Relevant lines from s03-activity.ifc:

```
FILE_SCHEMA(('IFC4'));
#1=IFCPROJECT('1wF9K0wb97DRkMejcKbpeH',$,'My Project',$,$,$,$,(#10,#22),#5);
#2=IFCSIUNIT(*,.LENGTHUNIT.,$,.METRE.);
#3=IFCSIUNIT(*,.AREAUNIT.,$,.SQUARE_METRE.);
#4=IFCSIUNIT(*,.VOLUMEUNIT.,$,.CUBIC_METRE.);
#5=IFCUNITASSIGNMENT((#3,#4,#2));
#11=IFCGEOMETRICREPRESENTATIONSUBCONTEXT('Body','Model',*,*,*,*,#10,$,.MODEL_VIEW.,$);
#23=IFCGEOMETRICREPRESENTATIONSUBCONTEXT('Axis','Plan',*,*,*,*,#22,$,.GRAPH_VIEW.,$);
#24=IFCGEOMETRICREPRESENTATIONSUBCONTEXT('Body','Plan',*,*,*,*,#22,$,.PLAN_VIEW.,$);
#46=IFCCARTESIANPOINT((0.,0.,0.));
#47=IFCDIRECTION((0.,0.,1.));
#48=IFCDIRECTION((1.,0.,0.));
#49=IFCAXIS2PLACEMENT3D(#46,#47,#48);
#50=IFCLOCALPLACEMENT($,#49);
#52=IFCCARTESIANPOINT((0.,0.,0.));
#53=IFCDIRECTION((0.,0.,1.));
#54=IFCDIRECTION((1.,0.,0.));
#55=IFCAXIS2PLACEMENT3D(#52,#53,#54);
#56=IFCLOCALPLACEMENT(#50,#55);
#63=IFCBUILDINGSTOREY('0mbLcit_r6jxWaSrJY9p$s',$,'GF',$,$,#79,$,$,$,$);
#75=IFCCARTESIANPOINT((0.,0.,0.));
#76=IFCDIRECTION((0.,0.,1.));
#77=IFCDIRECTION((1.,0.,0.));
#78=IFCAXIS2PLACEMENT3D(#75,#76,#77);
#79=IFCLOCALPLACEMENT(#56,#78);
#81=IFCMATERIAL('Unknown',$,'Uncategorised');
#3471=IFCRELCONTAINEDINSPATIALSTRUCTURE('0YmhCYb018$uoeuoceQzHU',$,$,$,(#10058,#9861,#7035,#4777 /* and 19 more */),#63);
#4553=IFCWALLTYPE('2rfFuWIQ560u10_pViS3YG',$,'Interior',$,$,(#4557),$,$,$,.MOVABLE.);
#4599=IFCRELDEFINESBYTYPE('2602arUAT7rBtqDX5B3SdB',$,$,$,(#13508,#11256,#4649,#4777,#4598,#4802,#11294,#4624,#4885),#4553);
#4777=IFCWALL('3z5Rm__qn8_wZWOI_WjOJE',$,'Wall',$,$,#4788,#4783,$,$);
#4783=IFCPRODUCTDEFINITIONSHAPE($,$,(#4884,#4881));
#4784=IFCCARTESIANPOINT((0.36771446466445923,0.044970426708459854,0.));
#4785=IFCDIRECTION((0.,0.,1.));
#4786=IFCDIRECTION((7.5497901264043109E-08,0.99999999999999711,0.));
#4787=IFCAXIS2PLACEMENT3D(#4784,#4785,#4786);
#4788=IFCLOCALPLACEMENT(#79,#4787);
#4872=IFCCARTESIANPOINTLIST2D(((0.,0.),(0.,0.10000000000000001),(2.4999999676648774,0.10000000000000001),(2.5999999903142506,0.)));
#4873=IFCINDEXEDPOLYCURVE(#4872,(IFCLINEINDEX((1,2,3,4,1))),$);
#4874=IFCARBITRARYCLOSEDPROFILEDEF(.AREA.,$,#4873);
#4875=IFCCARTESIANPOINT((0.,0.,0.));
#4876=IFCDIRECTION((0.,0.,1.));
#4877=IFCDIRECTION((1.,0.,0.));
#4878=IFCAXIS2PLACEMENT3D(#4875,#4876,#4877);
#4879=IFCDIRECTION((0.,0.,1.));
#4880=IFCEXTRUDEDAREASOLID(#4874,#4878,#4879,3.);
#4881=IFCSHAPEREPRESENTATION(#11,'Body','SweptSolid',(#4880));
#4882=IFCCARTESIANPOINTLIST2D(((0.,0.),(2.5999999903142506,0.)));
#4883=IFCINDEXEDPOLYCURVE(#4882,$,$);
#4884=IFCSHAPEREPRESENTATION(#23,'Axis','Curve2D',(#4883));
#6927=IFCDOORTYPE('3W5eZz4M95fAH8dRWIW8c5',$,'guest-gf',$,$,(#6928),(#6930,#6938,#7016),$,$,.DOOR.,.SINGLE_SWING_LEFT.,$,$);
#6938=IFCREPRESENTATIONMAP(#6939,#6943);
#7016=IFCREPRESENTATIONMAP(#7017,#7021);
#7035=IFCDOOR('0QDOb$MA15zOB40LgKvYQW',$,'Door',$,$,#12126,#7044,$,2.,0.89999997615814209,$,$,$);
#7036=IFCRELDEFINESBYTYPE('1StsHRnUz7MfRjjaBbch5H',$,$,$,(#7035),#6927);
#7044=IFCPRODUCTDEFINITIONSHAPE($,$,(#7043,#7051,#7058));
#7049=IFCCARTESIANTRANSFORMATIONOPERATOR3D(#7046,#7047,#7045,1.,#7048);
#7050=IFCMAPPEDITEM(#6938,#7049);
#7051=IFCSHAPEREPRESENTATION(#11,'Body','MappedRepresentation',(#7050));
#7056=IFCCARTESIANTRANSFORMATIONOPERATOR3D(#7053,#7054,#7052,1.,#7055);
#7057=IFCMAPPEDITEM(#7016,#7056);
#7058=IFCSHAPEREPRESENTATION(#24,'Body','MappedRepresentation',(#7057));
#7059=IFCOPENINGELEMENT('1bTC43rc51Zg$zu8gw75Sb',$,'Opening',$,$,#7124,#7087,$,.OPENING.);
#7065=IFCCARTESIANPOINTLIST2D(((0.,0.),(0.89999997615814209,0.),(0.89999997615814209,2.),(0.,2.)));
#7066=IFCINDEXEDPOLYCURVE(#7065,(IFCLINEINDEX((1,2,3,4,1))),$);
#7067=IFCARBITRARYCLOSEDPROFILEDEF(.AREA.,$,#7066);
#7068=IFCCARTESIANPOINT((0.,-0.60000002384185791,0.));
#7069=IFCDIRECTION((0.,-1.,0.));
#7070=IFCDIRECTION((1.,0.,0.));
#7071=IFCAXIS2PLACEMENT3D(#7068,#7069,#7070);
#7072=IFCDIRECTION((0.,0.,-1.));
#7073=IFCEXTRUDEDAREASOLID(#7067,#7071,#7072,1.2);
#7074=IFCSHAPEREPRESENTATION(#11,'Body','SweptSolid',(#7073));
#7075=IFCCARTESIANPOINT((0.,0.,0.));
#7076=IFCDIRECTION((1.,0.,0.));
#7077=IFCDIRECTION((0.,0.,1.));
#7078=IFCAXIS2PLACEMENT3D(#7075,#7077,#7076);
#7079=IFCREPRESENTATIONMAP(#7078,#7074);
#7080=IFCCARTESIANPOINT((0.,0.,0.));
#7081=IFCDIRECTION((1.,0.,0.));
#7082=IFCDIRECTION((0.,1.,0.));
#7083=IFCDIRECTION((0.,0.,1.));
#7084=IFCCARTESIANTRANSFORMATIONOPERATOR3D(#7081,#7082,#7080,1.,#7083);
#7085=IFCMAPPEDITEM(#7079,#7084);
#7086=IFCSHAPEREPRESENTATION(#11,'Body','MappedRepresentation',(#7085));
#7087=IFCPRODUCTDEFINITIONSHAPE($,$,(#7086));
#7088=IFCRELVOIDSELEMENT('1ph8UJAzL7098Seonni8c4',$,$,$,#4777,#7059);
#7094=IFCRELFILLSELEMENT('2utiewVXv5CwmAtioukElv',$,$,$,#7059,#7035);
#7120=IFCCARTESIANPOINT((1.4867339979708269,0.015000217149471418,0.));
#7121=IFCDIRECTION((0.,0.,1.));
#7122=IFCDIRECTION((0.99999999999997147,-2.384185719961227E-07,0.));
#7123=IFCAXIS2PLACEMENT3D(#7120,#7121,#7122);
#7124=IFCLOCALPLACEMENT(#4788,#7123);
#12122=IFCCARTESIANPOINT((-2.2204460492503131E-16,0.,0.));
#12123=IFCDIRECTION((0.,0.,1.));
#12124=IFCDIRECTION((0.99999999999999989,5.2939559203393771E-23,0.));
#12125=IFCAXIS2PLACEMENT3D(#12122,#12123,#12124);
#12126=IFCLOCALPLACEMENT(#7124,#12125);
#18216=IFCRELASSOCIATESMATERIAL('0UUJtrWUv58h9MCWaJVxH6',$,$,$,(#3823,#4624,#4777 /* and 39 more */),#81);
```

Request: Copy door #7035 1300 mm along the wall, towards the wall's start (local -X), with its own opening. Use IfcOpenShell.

```python
import ifcopenshell
import ifcopenshell.api.feature
import ifcopenshell.api.geometry
import ifcopenshell.api.root
import ifcopenshell.geom
import ifcopenshell.util.element
import ifcopenshell.util.placement
import ifcopenshell.util.shape
import ifcopenshell.util.unit

model = ifcopenshell.open("s03-activity.ifc")
unit_scale = ifcopenshell.util.unit.calculate_unit_scale(model)
settings = ifcopenshell.geom.settings()


def volume(element):
    """Net volume in cubic metres, openings subtracted."""
    shape = ifcopenshell.geom.create_shape(settings, element)
    return ifcopenshell.util.shape.get_volume(shape.geometry)


door = model.by_guid("0QDOb$MA15zOB40LgKvYQW")
opening = door.FillsVoids[0].RelatingOpeningElement
wall = opening.VoidsElements[0].RelatingBuildingElement
before = volume(wall)
shift = ifcopenshell.util.placement.get_local_placement(wall.ObjectPlacement)[:3, 0] * -1.3 / unit_scale

# copy_class copies the void relationship, type, container and properties, but no geometry.
new_opening = ifcopenshell.api.root.copy_class(model, product=opening)
new_opening.Representation = ifcopenshell.util.element.copy_deep(
    model, opening.Representation, exclude=["IfcGeometricRepresentationContext", "IfcRepresentationMap"]
)
new_door = ifcopenshell.api.root.copy_class(model, product=door)
new_door.Representation = ifcopenshell.util.element.copy_deep(
    model, door.Representation, exclude=["IfcGeometricRepresentationContext", "IfcRepresentationMap"]
)
ifcopenshell.api.feature.add_filling(model, opening=new_opening, element=new_door)

for old, new in ((opening, new_opening), (door, new_door)):
    matrix = ifcopenshell.util.placement.get_local_placement(old.ObjectPlacement)
    matrix[:3, 3] += shift
    ifcopenshell.api.geometry.edit_object_placement(model, product=new, matrix=matrix, is_si=False)

after = volume(wall)

print(f"wall volume {before:.3f} -> {after:.3f} m3")

model.write("s03-activity_v2.ifc")
```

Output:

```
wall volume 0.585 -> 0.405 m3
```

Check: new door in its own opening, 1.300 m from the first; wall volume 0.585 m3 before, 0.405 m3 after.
